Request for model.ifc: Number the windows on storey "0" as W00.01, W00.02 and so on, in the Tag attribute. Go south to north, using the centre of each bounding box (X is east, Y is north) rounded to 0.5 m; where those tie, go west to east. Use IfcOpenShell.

First a look at what the model holds.

```python
import ifcopenshell
import ifcopenshell.util.element
import ifcopenshell.util.placement

model = ifcopenshell.open("model.ifc")
print(model.schema)
storey = next(s for s in model.by_type("IfcBuildingStorey") if s.Name == "0")
windows = [e for e in ifcopenshell.util.element.get_decomposition(storey) if e.is_a("IfcWindow")]
for e in sorted(windows, key=lambda e: e.id()):
    origin = ifcopenshell.util.placement.get_local_placement(e.ObjectPlacement)[:3, 3]
    print(e.id(), e.Tag, e.Name, origin.round(2) + 0.0, sep=" | ")
```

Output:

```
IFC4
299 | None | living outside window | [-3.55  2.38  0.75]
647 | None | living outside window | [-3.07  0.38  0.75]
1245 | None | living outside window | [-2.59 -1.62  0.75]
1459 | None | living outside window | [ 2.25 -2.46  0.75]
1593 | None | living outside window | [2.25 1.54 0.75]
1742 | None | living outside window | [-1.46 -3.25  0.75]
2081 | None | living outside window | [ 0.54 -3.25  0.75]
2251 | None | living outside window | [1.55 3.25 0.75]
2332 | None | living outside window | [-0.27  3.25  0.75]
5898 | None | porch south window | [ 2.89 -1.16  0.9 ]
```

```python
import ifcopenshell
import ifcopenshell.geom
import ifcopenshell.util.element
import ifcopenshell.util.shape

model = ifcopenshell.open("model.ifc")
settings = ifcopenshell.geom.settings()
settings.set("use-world-coords", True)


def centre(element):
    shape = ifcopenshell.geom.create_shape(settings, element)
    return ifcopenshell.util.shape.get_bbox_centroid(shape.geometry)


storey = next(s for s in model.by_type("IfcBuildingStorey") if s.Name == "0")
windows = [e for e in ifcopenshell.util.element.get_decomposition(storey) if e.is_a("IfcWindow")]

# Insertion points can sit at a corner or the storey origin, so sort by the geometry (in metres).
centres = {e: centre(e) for e in windows}
windows.sort(key=lambda e: (round(centres[e][1] / 0.5), centres[e][0]))

for i, e in enumerate(windows, start=1):
    number = f"W00.{i:02d}"
    e.Tag = number
    print(e.id(), number)

model.write("model_rev.ifc")
```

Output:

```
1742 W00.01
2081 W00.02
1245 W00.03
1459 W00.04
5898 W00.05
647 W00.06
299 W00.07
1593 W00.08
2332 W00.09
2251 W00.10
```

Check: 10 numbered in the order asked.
